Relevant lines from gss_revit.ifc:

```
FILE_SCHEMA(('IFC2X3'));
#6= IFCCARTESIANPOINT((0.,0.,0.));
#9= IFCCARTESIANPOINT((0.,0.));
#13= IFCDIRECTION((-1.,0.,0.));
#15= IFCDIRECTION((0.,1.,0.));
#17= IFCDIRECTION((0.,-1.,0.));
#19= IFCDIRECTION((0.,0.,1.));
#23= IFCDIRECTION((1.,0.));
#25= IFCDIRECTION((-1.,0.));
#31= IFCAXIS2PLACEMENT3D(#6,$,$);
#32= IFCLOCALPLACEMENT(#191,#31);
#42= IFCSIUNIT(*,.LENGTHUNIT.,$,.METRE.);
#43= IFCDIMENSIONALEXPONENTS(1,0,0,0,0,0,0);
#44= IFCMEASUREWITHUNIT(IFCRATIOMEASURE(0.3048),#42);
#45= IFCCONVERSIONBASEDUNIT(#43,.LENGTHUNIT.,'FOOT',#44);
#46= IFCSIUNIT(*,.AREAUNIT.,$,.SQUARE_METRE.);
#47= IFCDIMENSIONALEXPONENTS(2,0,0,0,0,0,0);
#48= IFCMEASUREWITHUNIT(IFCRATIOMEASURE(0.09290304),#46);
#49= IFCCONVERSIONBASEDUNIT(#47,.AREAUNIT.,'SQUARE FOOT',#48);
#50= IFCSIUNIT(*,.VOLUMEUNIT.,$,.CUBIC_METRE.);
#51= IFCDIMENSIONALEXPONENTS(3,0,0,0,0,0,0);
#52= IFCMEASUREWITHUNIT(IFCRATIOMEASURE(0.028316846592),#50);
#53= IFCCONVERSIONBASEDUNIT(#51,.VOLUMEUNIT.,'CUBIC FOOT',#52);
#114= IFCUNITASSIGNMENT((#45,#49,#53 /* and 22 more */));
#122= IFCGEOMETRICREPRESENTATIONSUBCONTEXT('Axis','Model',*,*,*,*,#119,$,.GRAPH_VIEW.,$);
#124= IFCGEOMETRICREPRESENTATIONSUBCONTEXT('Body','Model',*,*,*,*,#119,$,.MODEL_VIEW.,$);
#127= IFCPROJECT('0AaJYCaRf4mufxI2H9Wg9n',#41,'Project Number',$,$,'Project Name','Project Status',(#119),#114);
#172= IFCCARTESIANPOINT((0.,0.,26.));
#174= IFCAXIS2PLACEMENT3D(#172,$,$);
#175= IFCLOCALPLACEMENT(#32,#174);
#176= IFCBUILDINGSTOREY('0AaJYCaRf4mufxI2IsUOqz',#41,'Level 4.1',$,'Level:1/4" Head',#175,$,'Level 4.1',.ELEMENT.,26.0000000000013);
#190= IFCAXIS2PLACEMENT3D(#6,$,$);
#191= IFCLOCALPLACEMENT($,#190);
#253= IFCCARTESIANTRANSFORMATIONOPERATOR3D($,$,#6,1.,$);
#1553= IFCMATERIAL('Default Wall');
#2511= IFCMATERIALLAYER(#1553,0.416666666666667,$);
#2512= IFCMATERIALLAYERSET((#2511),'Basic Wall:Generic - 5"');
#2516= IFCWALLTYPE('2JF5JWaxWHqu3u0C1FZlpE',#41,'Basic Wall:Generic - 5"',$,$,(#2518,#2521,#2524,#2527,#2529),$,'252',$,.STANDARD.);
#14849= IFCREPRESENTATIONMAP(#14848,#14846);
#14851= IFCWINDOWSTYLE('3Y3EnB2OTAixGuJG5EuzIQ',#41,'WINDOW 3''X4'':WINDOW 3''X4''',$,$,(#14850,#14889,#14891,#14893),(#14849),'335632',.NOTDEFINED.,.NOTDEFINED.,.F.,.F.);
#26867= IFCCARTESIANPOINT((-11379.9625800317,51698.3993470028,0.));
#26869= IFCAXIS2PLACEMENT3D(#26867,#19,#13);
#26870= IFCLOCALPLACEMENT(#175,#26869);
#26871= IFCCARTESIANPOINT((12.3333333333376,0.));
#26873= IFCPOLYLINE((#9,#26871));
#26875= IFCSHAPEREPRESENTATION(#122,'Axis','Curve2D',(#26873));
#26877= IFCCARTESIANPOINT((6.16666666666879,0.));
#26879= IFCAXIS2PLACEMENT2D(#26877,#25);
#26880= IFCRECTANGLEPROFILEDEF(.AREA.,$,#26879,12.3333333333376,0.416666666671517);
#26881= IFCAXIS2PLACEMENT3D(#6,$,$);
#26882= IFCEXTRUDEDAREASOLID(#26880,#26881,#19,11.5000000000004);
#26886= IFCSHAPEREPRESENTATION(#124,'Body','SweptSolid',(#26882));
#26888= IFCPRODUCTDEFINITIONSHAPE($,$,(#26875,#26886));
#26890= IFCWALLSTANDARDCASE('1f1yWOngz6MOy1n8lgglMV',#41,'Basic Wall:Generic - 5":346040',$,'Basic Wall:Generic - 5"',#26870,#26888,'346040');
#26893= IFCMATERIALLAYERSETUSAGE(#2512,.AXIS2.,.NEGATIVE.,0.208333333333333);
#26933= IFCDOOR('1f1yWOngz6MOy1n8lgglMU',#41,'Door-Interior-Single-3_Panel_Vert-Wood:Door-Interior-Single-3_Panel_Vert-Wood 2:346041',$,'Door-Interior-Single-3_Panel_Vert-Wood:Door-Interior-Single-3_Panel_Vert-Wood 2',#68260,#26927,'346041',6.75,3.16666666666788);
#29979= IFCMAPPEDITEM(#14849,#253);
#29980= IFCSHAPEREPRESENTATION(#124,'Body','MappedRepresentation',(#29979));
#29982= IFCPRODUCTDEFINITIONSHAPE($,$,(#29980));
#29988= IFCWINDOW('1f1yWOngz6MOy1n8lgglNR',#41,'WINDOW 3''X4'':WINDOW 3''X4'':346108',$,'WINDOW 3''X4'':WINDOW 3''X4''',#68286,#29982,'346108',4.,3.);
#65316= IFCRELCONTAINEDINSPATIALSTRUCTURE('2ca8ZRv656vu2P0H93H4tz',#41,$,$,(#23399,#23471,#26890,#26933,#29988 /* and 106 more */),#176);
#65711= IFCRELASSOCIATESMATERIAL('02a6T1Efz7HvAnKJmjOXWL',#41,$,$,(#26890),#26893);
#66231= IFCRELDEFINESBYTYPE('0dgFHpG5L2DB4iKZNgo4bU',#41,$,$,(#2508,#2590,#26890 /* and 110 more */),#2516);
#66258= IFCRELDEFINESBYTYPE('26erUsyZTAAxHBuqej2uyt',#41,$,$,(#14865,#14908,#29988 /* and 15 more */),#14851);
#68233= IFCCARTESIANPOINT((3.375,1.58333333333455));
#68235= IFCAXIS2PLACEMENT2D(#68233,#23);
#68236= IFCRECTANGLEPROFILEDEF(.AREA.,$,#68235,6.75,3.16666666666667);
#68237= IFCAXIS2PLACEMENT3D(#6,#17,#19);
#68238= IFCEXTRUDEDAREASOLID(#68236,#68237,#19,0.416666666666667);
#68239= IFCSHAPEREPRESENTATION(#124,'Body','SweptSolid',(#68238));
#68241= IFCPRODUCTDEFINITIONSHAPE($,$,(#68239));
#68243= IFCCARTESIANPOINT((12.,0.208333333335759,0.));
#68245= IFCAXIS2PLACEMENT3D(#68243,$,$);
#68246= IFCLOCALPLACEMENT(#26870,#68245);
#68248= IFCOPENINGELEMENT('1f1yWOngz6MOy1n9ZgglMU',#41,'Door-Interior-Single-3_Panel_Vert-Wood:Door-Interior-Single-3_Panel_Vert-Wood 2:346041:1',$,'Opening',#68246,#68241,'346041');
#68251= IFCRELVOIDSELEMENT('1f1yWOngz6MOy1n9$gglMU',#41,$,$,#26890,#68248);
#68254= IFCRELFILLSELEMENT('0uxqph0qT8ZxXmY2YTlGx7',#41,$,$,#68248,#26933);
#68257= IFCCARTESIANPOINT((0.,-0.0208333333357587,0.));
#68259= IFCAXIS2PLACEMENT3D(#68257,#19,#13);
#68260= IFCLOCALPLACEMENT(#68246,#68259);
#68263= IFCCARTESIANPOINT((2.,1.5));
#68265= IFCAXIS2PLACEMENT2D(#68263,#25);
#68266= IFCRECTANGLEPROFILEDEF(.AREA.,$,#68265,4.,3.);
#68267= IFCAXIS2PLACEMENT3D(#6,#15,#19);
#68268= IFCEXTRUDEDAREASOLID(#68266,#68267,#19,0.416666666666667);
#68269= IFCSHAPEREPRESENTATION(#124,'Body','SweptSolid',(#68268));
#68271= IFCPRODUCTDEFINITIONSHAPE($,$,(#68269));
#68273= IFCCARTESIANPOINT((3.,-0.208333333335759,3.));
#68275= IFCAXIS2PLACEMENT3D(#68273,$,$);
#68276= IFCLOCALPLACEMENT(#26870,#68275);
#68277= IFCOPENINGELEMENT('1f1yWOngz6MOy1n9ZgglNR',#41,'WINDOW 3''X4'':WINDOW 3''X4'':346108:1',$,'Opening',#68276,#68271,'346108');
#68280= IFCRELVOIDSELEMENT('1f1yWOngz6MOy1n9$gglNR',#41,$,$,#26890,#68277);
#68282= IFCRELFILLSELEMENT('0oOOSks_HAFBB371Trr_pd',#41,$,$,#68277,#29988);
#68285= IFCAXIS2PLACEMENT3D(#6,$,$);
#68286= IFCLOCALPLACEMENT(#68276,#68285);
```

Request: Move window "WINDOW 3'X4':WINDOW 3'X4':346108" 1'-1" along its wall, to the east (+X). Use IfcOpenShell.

```python
import ifcopenshell
import ifcopenshell.api.geometry
import ifcopenshell.util.placement
import ifcopenshell.util.unit

model = ifcopenshell.open("gss_revit.ifc")
unit_scale = ifcopenshell.util.unit.calculate_unit_scale(model)

window = model.by_guid("1f1yWOngz6MOy1n8lgglNR")
opening = window.FillsVoids[0].RelatingOpeningElement
wall = opening.VoidsElements[0].RelatingBuildingElement

wall_matrix = ifcopenshell.util.placement.get_local_placement(wall.ObjectPlacement)
shift = wall_matrix[:3, 0] * -13 * 0.0254 / unit_scale
before = ifcopenshell.util.placement.get_local_placement(window.ObjectPlacement)[:3, 3].copy()

# The window is placed relative to its opening, so it follows when the opening moves.
matrix = ifcopenshell.util.placement.get_local_placement(opening.ObjectPlacement)
matrix[:3, 3] += shift
ifcopenshell.api.geometry.edit_object_placement(
    model, product=opening, matrix=matrix, is_si=False, should_transform_children=True
)

after = ifcopenshell.util.placement.get_local_placement(window.ObjectPlacement)[:3, 3]
print("window moved by", (after - before).round(3) + 0.0)

model.write("gss_revit_edited.ifc")
```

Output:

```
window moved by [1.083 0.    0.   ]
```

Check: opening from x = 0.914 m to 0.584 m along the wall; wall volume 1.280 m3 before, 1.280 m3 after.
